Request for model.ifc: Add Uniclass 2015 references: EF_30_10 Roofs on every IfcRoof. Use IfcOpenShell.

First a look at what the model holds.

```python
import ifcopenshell

model = ifcopenshell.open("model.ifc")
print(model.schema)
print("classifications:", [c.Name for c in model.by_type("IfcClassification")])
for ifc_class in ("IfcDoor", "IfcRoof", "IfcStair", "IfcWall", "IfcWindow"):
    print(ifc_class, len(model.by_type(ifc_class)))
```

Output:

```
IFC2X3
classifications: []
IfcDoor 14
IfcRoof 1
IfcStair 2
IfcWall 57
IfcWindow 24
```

```python
import ifcopenshell
import ifcopenshell.api.classification

model = ifcopenshell.open("model.ifc")

# IFC2X3 requires Source and Edition and has no link from the project to the system.
system = model.create_entity("IfcClassification", Source="NBS", Edition="2015", Name="Uniclass 2015")

codes = {
    "IfcRoof": ("EF_30_10", "Roofs"),
}
for ifc_class, (code, name) in codes.items():
    products = model.by_type(ifc_class)
    ifcopenshell.api.classification.add_reference(
        model, products=products, classification=system, identification=code, name=name
    )
    print(code, len(products))

model.write("model_v2.ifc")
```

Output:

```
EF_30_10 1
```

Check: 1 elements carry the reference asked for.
